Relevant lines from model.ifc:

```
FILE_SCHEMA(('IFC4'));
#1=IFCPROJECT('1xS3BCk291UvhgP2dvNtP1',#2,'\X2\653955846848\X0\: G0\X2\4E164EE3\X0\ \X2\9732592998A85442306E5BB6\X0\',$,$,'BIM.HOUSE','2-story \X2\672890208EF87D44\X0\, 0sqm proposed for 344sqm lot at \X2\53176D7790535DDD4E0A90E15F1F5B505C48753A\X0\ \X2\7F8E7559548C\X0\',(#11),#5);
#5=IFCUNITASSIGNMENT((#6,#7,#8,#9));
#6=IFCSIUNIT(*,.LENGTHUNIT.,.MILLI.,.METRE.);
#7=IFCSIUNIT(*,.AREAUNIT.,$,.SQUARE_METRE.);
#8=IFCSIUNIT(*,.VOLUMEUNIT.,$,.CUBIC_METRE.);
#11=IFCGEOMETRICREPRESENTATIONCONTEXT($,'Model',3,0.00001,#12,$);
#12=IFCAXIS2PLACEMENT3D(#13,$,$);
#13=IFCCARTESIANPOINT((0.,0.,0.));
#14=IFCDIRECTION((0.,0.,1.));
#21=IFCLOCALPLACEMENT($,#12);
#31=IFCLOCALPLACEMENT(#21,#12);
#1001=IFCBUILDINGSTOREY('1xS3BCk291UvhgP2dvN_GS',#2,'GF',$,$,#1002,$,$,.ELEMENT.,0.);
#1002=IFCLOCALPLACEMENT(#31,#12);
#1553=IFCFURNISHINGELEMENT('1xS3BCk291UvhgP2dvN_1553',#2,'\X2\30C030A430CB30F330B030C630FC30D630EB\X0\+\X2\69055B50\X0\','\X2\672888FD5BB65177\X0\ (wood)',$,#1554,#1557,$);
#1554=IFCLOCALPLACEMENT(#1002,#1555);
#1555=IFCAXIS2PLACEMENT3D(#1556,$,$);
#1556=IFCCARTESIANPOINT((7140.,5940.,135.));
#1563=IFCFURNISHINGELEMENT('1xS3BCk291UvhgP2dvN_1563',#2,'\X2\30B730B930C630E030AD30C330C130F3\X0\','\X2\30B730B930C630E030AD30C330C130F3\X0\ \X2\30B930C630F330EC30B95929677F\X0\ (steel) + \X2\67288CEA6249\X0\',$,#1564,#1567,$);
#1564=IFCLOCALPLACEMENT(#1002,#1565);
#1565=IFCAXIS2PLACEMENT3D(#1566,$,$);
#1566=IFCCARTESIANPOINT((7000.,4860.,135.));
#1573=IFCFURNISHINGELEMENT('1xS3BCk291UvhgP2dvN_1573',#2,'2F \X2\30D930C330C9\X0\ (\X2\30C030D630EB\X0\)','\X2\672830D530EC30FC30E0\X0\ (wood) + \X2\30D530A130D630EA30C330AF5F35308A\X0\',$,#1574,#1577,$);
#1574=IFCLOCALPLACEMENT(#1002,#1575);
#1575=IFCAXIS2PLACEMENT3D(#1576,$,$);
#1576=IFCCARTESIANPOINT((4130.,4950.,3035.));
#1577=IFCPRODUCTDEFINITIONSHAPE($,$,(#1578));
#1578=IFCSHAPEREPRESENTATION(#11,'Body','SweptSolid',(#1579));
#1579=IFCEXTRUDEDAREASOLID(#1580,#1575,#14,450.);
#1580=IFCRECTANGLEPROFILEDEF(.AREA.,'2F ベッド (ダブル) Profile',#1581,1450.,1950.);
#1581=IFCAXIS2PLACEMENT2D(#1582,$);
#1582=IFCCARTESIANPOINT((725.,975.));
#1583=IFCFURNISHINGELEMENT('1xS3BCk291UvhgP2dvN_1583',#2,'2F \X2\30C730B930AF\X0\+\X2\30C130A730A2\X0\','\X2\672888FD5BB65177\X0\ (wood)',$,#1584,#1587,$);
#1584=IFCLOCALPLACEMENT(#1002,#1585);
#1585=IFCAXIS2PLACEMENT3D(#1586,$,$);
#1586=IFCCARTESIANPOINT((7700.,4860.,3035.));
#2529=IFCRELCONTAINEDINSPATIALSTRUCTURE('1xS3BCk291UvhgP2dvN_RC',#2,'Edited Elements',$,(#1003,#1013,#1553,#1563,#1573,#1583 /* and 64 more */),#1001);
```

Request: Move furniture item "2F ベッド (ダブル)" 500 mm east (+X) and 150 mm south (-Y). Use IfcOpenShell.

```python
import ifcopenshell
import ifcopenshell.api.geometry
import ifcopenshell.util.placement

model = ifcopenshell.open("model.ifc")

item = model.by_guid("1xS3BCk291UvhgP2dvN_1573")
matrix = ifcopenshell.util.placement.get_local_placement(item.ObjectPlacement)
matrix[0, 3] += 500.0
matrix[1, 3] -= 150.0
ifcopenshell.api.geometry.edit_object_placement(model, product=item, matrix=matrix, is_si=False)

print(ifcopenshell.util.placement.get_local_placement(item.ObjectPlacement).round(3) + 0.0)

model.write("model-out.ifc")
```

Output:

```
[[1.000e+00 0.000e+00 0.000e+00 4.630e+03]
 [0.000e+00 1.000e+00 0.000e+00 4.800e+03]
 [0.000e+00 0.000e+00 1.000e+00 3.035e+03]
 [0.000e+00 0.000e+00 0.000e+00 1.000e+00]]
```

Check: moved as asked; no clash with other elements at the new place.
